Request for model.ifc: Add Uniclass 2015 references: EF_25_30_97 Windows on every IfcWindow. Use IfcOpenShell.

First a look at what the model holds.

```python
import ifcopenshell

model = ifcopenshell.open("model.ifc")
print(model.schema)
print("classifications:", [c.Name for c in model.by_type("IfcClassification")])
for ifc_class in ("IfcDoor", "IfcRoof", "IfcStair", "IfcWall", "IfcWindow"):
    print(ifc_class, len(model.by_type(ifc_class)))
```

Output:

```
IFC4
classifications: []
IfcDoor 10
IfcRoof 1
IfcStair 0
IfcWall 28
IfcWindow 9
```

```python
import ifcopenshell
import ifcopenshell.api.classification

model = ifcopenshell.open("model.ifc")

system = ifcopenshell.api.classification.add_classification(model, classification="Uniclass 2015")

codes = {
    "IfcWindow": ("EF_25_30_97", "Windows"),
}
for ifc_class, (code, name) in codes.items():
    products = model.by_type(ifc_class)
    ifcopenshell.api.classification.add_reference(
        model, products=products, classification=system, identification=code, name=name
    )
    print(code, len(products))

model.write("model-out.ifc")
```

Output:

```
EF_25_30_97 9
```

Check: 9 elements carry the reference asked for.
